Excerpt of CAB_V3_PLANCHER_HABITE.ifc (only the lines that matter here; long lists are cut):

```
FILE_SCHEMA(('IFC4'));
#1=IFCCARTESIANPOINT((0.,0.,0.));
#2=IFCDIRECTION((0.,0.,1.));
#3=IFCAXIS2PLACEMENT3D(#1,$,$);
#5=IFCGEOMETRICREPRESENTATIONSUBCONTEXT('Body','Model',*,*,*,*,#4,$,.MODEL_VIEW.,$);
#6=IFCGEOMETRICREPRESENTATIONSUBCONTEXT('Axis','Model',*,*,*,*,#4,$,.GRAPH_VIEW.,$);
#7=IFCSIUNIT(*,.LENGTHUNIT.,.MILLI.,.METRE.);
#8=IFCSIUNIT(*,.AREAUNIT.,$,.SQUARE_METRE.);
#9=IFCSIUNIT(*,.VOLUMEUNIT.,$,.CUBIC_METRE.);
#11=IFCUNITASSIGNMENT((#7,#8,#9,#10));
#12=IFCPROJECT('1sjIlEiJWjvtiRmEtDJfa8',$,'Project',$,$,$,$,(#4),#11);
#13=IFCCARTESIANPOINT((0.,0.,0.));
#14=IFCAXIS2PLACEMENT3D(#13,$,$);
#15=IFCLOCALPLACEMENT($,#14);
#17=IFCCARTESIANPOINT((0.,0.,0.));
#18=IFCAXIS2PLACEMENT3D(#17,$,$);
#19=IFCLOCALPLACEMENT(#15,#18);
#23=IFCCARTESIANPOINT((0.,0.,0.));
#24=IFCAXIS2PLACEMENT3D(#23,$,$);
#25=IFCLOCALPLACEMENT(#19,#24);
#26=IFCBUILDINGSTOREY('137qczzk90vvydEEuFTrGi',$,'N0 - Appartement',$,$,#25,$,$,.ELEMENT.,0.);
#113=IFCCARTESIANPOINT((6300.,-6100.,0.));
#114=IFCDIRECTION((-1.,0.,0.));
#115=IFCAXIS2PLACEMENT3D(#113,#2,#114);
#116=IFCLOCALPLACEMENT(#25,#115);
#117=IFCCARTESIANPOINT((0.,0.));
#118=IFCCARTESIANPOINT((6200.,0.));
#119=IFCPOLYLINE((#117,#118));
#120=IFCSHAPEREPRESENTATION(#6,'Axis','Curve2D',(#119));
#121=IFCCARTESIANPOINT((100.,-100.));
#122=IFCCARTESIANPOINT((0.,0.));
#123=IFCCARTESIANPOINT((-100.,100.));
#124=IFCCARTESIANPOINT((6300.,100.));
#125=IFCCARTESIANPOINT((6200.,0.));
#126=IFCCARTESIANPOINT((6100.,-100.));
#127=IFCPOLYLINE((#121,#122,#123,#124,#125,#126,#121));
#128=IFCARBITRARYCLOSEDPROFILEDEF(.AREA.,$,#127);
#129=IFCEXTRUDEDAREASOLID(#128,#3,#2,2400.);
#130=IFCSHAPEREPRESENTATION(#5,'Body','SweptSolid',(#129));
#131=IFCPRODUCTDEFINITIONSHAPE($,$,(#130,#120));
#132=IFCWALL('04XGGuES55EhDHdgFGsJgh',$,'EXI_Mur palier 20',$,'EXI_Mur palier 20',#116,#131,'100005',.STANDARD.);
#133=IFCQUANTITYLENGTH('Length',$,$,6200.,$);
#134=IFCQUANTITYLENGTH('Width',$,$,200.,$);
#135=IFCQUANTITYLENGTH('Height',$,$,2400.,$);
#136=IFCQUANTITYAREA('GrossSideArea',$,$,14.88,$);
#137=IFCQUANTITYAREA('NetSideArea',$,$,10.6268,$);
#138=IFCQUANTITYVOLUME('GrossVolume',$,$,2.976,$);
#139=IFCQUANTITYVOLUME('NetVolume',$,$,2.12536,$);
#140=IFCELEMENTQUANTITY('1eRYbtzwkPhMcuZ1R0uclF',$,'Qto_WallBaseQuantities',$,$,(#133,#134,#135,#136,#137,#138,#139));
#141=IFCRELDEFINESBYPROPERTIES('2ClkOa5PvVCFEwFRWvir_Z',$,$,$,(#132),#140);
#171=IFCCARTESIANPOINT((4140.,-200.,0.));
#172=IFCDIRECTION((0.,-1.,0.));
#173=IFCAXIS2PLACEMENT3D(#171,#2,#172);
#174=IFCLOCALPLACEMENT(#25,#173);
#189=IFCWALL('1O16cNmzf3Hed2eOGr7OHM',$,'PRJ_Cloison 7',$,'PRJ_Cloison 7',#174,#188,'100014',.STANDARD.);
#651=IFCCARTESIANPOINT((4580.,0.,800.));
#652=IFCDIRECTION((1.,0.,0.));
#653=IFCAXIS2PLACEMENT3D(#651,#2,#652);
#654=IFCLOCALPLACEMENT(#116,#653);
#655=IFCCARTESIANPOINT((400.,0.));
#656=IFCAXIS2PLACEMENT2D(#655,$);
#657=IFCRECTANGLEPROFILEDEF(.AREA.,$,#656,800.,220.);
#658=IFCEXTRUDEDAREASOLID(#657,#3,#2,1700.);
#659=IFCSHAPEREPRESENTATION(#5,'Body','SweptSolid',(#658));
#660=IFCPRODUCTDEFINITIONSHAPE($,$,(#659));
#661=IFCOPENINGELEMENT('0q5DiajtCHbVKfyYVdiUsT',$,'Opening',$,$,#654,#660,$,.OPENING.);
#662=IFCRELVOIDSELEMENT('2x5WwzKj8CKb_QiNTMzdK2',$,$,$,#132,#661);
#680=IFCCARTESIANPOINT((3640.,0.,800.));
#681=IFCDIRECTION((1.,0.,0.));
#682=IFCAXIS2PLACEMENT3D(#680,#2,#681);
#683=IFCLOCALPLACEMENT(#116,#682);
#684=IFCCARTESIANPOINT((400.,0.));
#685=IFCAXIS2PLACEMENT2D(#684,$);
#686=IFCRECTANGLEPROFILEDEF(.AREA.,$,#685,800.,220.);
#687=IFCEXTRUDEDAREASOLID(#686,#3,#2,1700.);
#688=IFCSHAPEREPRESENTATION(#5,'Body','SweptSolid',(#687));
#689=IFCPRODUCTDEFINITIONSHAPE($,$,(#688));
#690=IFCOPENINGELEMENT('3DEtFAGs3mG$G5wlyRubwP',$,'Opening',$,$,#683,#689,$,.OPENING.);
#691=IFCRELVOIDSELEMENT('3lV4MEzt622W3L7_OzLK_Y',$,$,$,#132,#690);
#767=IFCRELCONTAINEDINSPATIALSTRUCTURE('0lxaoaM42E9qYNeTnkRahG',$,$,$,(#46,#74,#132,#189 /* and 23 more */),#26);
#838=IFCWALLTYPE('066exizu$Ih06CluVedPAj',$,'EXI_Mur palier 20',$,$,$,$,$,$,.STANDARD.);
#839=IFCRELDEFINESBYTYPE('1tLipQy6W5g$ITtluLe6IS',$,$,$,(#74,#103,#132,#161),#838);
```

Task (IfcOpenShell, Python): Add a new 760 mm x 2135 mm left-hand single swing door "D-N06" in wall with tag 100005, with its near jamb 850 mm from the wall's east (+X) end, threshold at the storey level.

```python
import numpy as np
import ifcopenshell
import ifcopenshell.api.feature
import ifcopenshell.api.geometry
import ifcopenshell.api.pset
import ifcopenshell.api.root
import ifcopenshell.api.spatial
import ifcopenshell.geom
import ifcopenshell.util.element
import ifcopenshell.util.placement
import ifcopenshell.util.representation
import ifcopenshell.util.shape
import ifcopenshell.util.unit

model = ifcopenshell.open("CAB_V3_PLANCHER_HABITE.ifc")
unit_scale = ifcopenshell.util.unit.calculate_unit_scale(model)
area_scale = ifcopenshell.util.unit.calculate_unit_scale(model, "AREAUNIT")
volume_scale = ifcopenshell.util.unit.calculate_unit_scale(model, "VOLUMEUNIT")
settings = ifcopenshell.geom.settings()


def volume(element):
    """Net volume in cubic metres, openings subtracted."""
    shape = ifcopenshell.geom.create_shape(settings, element)
    return ifcopenshell.util.shape.get_volume(shape.geometry)


wall = model.by_guid("04XGGuES55EhDHdgFGsJgh")
storey = ifcopenshell.util.element.get_container(wall, ifc_class="IfcBuildingStorey")
context = ifcopenshell.util.representation.get_context(model, "Model", "Body", "MODEL_VIEW")
before = volume(wall)

width, height, from_end, sill = 0.76, 2.135, 0.85, 0.0  # metres

# The wall runs along its own X axis, and the end named is its -X end.
wall_shape = ifcopenshell.geom.create_shape(settings, wall)
x, y, z = ifcopenshell.util.shape.get_vertices(wall_shape.geometry).T
start = x.min() + from_end
face, thickness = float(y.min()), float(y.max() - y.min())
wall_matrix = ifcopenshell.util.placement.get_local_placement(wall.ObjectPlacement)
level = ifcopenshell.util.placement.get_local_placement(storey.ObjectPlacement)[2, 3]


def in_wall(x, y):
    """Placement at x, y metres in the wall's axes, at sill height."""
    matrix = wall_matrix.copy()
    matrix[:, 3] = wall_matrix @ np.array([x / unit_scale, y / unit_scale, 0.0, 1.0])
    matrix[2, 3] = level + sill / unit_scale
    return matrix


# Opening: a box that overshoots both wall faces by 50 mm.
opening = ifcopenshell.api.root.create_entity(model, ifc_class="IfcOpeningElement", predefined_type="OPENING")
box = ifcopenshell.api.geometry.add_wall_representation(
    model, context=context, length=width, height=height, thickness=thickness + 0.1
)
ifcopenshell.api.geometry.assign_representation(model, product=opening, representation=box)
ifcopenshell.api.geometry.edit_object_placement(model, product=opening, matrix=in_wall(start, face - 0.05), is_si=False)
ifcopenshell.api.feature.add_feature(model, feature=opening, element=wall)

door = ifcopenshell.api.root.create_entity(model, ifc_class="IfcDoor", name="D-N06", predefined_type="DOOR")
door.OverallWidth, door.OverallHeight = width / unit_scale, height / unit_scale
door.OperationType = "SINGLE_SWING_LEFT"
body = ifcopenshell.api.geometry.add_door_representation(
    model,
    context=context,
    overall_width=door.OverallWidth,
    overall_height=door.OverallHeight,
    operation_type="SINGLE_SWING_LEFT",
    lining_properties={"LiningDepth": thickness / unit_scale, "ThresholdDepth": thickness / unit_scale},
)
ifcopenshell.api.geometry.assign_representation(model, product=door, representation=body)
ifcopenshell.api.spatial.assign_container(model, products=[door], relating_structure=storey)
ifcopenshell.api.feature.add_filling(model, opening=opening, element=door)

# The lining spans the wall, so the door starts at the wall face.
ifcopenshell.api.geometry.edit_object_placement(model, product=door, matrix=in_wall(start, face), is_si=False)

after = volume(wall)

# Update the wall's stored quantities.
qto = model.by_id(ifcopenshell.util.element.get_pset(wall, "Qto_WallBaseQuantities", should_inherit=False)["id"])
ifcopenshell.api.pset.edit_qto(model, qto=qto, properties={
    "NetSideArea": after / thickness / area_scale,
    "NetVolume": after / volume_scale,
})

print(f"wall volume {before:.3f} -> {after:.3f} m3")

model.write("CAB_V3_PLANCHER_HABITE-out.ifc")
```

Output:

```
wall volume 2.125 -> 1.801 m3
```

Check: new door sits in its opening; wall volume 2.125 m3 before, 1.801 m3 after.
